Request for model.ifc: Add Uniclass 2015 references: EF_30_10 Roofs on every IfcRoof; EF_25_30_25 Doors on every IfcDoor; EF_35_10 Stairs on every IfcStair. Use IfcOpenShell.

First a look at what the model holds.

```python
import ifcopenshell

model = ifcopenshell.open("model.ifc")
print(model.schema)
print("classifications:", [c.Name for c in model.by_type("IfcClassification")])
for ifc_class in ("IfcDoor", "IfcRoof", "IfcStair", "IfcWall", "IfcWindow"):
    print(ifc_class, len(model.by_type(ifc_class)))
```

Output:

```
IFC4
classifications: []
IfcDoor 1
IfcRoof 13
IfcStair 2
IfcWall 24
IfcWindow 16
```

```python
import ifcopenshell
import ifcopenshell.api.classification

model = ifcopenshell.open("model.ifc")

system = ifcopenshell.api.classification.add_classification(model, classification="Uniclass 2015")

codes = {
    "IfcRoof": ("EF_30_10", "Roofs"),
    "IfcDoor": ("EF_25_30_25", "Doors"),
    "IfcStair": ("EF_35_10", "Stairs"),
}
for ifc_class, (code, name) in codes.items():
    products = model.by_type(ifc_class)
    ifcopenshell.api.classification.add_reference(
        model, products=products, classification=system, identification=code, name=name
    )
    print(code, len(products))

model.write("model_rev.ifc")
```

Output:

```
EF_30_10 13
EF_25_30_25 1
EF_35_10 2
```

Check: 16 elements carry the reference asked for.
